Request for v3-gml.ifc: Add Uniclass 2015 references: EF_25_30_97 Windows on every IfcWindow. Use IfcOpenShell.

First a look at what the model holds.

```python
import ifcopenshell

model = ifcopenshell.open("v3-gml.ifc")
print(model.schema)
print("classifications:", [c.Name for c in model.by_type("IfcClassification")])
for ifc_class in ("IfcDoor", "IfcRoof", "IfcStair", "IfcWall", "IfcWindow"):
    print(ifc_class, len(model.by_type(ifc_class)))
```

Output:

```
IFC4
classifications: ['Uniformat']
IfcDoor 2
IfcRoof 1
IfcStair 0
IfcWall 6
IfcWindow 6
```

```python
import ifcopenshell
import ifcopenshell.api.classification

model = ifcopenshell.open("v3-gml.ifc")

system = ifcopenshell.api.classification.add_classification(model, classification="Uniclass 2015")

codes = {
    "IfcWindow": ("EF_25_30_97", "Windows"),
}
for ifc_class, (code, name) in codes.items():
    products = model.by_type(ifc_class)
    ifcopenshell.api.classification.add_reference(
        model, products=products, classification=system, identification=code, name=name
    )
    print(code, len(products))

model.write("v3-gml_updated.ifc")
```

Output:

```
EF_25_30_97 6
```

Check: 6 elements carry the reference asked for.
